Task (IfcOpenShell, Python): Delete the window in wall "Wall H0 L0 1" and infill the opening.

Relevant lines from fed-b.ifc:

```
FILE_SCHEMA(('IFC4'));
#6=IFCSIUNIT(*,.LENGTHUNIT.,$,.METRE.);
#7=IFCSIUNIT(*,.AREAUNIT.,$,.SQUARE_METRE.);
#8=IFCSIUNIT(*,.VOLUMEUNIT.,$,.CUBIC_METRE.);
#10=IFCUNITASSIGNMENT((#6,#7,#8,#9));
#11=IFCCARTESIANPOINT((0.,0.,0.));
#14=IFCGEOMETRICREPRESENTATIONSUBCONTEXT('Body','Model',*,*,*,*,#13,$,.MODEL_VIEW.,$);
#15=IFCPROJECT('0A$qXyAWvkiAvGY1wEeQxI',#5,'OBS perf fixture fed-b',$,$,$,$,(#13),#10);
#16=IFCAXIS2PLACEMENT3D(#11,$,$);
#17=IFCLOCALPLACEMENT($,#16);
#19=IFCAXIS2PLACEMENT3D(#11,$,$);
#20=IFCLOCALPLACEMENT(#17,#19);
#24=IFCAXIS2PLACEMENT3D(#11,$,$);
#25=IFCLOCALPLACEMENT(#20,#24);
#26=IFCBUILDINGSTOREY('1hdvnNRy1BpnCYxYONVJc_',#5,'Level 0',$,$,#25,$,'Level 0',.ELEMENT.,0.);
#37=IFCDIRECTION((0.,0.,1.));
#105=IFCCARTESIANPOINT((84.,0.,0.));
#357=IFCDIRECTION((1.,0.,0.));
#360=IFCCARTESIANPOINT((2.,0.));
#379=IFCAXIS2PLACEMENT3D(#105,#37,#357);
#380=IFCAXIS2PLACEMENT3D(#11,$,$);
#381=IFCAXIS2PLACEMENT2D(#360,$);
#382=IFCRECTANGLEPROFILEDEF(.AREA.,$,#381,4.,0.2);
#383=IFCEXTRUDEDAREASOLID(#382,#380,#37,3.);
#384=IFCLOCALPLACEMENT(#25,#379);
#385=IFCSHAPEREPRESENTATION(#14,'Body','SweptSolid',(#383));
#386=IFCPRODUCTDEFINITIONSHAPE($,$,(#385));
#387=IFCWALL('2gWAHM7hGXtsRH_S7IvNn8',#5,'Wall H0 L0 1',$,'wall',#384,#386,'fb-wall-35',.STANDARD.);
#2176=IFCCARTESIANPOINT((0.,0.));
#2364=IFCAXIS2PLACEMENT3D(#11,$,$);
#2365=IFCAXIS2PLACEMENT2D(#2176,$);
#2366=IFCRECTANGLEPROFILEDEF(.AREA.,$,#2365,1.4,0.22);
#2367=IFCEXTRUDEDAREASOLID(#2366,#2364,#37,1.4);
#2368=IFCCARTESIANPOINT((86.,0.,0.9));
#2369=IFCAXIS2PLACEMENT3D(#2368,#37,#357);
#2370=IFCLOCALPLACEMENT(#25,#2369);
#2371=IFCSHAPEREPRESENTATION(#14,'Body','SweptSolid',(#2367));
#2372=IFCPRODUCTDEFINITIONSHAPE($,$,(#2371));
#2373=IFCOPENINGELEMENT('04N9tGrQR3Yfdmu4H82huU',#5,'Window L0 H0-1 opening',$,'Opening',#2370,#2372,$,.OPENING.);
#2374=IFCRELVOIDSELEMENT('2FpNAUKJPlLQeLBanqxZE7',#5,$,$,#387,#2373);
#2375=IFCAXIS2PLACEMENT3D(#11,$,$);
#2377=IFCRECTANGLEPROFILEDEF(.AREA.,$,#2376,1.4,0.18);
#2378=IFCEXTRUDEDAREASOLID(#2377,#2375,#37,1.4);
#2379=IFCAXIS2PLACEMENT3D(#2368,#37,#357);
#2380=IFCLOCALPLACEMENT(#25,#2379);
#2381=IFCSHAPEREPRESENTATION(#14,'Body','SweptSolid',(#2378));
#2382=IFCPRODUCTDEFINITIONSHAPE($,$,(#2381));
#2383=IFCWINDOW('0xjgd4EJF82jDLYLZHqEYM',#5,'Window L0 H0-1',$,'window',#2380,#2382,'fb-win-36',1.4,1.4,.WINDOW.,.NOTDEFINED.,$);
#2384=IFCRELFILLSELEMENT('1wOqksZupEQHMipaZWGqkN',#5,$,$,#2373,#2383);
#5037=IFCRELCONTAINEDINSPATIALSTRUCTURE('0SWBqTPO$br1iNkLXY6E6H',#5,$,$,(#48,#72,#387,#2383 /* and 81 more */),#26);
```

```python
import ifcopenshell
import ifcopenshell.api.feature
import ifcopenshell.api.root
import ifcopenshell.geom
import ifcopenshell.util.shape

model = ifcopenshell.open("fed-b.ifc")
settings = ifcopenshell.geom.settings()


def volume(element):
    """Net volume in cubic metres, openings subtracted."""
    shape = ifcopenshell.geom.create_shape(settings, element)
    return ifcopenshell.util.shape.get_volume(shape.geometry)


window = model.by_guid("0xjgd4EJF82jDLYLZHqEYM")
opening = window.FillsVoids[0].RelatingOpeningElement
wall = opening.VoidsElements[0].RelatingBuildingElement
before = volume(wall)

ifcopenshell.api.root.remove_product(model, product=window)
ifcopenshell.api.feature.remove_feature(model, feature=opening)

after = volume(wall)

print(f"wall volume {before:.3f} -> {after:.3f} m3")

model.write("fed-b_edited.ifc")
```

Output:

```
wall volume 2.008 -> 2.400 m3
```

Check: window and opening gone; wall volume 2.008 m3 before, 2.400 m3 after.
